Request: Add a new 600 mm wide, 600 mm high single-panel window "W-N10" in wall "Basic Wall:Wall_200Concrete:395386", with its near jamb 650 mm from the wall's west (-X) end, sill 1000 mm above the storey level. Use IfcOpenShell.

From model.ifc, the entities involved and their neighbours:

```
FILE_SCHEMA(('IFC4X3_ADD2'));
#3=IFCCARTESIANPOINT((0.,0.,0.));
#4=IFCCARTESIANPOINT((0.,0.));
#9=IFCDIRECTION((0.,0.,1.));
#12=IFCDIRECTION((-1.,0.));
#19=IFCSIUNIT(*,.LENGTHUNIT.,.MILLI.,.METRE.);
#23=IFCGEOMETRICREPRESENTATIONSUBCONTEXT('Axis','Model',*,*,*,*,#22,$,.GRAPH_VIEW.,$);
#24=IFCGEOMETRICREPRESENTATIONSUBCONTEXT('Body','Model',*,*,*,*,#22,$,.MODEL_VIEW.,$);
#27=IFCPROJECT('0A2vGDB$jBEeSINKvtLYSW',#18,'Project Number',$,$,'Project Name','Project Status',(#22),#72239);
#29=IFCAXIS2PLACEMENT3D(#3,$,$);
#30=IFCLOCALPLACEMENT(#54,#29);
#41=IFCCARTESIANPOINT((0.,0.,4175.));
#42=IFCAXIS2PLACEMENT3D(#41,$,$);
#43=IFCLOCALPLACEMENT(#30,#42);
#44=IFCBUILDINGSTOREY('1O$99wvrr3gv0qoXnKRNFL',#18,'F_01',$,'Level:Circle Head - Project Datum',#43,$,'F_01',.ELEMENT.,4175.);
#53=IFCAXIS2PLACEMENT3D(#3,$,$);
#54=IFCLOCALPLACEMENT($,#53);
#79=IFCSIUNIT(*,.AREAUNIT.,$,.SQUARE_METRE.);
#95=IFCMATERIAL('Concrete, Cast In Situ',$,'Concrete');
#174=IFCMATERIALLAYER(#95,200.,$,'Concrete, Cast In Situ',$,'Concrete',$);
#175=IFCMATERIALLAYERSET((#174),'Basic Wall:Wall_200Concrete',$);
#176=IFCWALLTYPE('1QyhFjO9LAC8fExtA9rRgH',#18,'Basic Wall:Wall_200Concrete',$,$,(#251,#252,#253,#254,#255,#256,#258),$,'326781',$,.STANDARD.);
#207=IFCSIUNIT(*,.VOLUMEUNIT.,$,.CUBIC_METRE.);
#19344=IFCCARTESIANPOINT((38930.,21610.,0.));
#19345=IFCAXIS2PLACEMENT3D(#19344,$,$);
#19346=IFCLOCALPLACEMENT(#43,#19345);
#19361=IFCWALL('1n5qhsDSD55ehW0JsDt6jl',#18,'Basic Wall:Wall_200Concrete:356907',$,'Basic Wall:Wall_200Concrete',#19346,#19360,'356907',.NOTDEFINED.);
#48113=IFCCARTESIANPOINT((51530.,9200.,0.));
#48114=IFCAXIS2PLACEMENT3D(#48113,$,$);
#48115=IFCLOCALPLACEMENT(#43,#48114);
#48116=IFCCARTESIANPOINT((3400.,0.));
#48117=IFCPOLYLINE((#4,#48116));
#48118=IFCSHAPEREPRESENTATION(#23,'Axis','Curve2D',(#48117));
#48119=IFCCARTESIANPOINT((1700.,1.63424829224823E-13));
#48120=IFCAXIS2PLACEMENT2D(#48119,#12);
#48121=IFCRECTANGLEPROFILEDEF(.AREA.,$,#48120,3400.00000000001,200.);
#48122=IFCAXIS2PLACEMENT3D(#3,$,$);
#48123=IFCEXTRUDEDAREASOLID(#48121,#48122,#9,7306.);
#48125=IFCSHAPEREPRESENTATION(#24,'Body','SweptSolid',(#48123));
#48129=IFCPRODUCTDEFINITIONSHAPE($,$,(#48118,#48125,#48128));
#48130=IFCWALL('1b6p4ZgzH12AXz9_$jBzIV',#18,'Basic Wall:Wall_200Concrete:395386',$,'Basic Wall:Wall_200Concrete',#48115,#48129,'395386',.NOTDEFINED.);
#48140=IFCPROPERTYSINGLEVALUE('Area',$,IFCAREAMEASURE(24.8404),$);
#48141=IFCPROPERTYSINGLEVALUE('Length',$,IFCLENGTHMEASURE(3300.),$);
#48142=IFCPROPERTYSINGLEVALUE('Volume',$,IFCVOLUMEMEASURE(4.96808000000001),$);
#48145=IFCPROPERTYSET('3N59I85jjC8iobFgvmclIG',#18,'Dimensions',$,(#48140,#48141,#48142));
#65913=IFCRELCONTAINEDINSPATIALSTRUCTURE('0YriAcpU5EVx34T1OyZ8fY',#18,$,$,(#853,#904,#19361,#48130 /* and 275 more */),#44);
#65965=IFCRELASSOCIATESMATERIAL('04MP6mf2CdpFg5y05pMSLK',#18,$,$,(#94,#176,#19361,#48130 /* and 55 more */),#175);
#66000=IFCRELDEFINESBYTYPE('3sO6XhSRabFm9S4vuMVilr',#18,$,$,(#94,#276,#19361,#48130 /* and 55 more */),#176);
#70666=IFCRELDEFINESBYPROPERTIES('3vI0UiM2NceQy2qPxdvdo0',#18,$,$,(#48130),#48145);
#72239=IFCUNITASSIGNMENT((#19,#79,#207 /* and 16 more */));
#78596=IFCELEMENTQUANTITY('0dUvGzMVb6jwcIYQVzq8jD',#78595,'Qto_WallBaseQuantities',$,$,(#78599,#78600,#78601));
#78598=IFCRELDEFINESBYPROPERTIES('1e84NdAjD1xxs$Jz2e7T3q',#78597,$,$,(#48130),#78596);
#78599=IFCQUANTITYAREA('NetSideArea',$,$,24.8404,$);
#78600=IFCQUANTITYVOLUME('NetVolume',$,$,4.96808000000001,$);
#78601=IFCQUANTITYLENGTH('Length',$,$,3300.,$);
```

```python
import numpy as np
import ifcopenshell
import ifcopenshell.api.feature
import ifcopenshell.api.geometry
import ifcopenshell.api.pset
import ifcopenshell.api.root
import ifcopenshell.api.spatial
import ifcopenshell.geom
import ifcopenshell.util.element
import ifcopenshell.util.placement
import ifcopenshell.util.representation
import ifcopenshell.util.shape
import ifcopenshell.util.unit

model = ifcopenshell.open("model.ifc")
unit_scale = ifcopenshell.util.unit.calculate_unit_scale(model)
area_scale = ifcopenshell.util.unit.calculate_unit_scale(model, "AREAUNIT")
volume_scale = ifcopenshell.util.unit.calculate_unit_scale(model, "VOLUMEUNIT")
settings = ifcopenshell.geom.settings()


def volume(element):
    """Net volume in cubic metres, openings subtracted."""
    shape = ifcopenshell.geom.create_shape(settings, element)
    return ifcopenshell.util.shape.get_volume(shape.geometry)


wall = model.by_id(48130)
storey = ifcopenshell.util.element.get_container(wall, ifc_class="IfcBuildingStorey")
context = ifcopenshell.util.representation.get_context(model, "Model", "Body", "MODEL_VIEW")
before = volume(wall)

width, height, from_end, sill = 0.6, 0.6, 0.65, 1  # metres

# The wall runs along its own X axis, and the end named is its -X end.
wall_shape = ifcopenshell.geom.create_shape(settings, wall)
x, y, z = ifcopenshell.util.shape.get_vertices(wall_shape.geometry).T
start = x.min() + from_end
face, thickness = float(y.min()), float(y.max() - y.min())
wall_matrix = ifcopenshell.util.placement.get_local_placement(wall.ObjectPlacement)
level = ifcopenshell.util.placement.get_local_placement(storey.ObjectPlacement)[2, 3]


def in_wall(x, y):
    """Placement at x, y metres in the wall's axes, at sill height."""
    matrix = wall_matrix.copy()
    matrix[:, 3] = wall_matrix @ np.array([x / unit_scale, y / unit_scale, 0.0, 1.0])
    matrix[2, 3] = level + sill / unit_scale
    return matrix


# Opening: a box that overshoots both wall faces by 50 mm.
opening = ifcopenshell.api.root.create_entity(model, ifc_class="IfcOpeningElement", predefined_type="OPENING")
box = ifcopenshell.api.geometry.add_wall_representation(
    model, context=context, length=width, height=height, thickness=thickness + 0.1
)
ifcopenshell.api.geometry.assign_representation(model, product=opening, representation=box)
ifcopenshell.api.geometry.edit_object_placement(model, product=opening, matrix=in_wall(start, face - 0.05), is_si=False)
ifcopenshell.api.feature.add_feature(model, feature=opening, element=wall)

window = ifcopenshell.api.root.create_entity(model, ifc_class="IfcWindow", name="W-N10", predefined_type="WINDOW")
window.OverallWidth, window.OverallHeight = width / unit_scale, height / unit_scale
window.PartitioningType = "SINGLE_PANEL"
body = ifcopenshell.api.geometry.add_window_representation(
    model,
    context=context,
    overall_width=window.OverallWidth,
    overall_height=window.OverallHeight,
    partition_type="SINGLE_PANEL",
)
ifcopenshell.api.geometry.assign_representation(model, product=window, representation=body)
ifcopenshell.api.spatial.assign_container(model, products=[window], relating_structure=storey)
ifcopenshell.api.feature.add_filling(model, opening=opening, element=window)

# Centre the window in the wall's thickness.
ifcopenshell.api.geometry.edit_object_placement(model, product=window, matrix=in_wall(start, face), is_si=False)
window_shape = ifcopenshell.geom.create_shape(settings, window)
depth = ifcopenshell.util.shape.get_vertices(window_shape.geometry)[:, 1]
offset = face + thickness / 2 - (depth.min() + depth.max()) / 2
ifcopenshell.api.geometry.edit_object_placement(model, product=window, matrix=in_wall(start, offset), is_si=False)

after = volume(wall)

# Update the wall's stored quantities.
pset = model.by_id(ifcopenshell.util.element.get_pset(wall, "Dimensions", should_inherit=False)["id"])
ifcopenshell.api.pset.edit_pset(model, pset=pset, properties={
    "Area": model.create_entity("IfcAreaMeasure", after / thickness / area_scale),
    "Volume": model.create_entity("IfcVolumeMeasure", after / volume_scale),
})
qto = model.by_id(ifcopenshell.util.element.get_pset(wall, "Qto_WallBaseQuantities", should_inherit=False)["id"])
ifcopenshell.api.pset.edit_qto(model, qto=qto, properties={
    "NetSideArea": after / thickness / area_scale,
    "NetVolume": after / volume_scale,
})

print(f"wall volume {before:.3f} -> {after:.3f} m3")

model.write("model-out.ifc")
```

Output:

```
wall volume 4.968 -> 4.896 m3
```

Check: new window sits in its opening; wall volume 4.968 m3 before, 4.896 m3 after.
